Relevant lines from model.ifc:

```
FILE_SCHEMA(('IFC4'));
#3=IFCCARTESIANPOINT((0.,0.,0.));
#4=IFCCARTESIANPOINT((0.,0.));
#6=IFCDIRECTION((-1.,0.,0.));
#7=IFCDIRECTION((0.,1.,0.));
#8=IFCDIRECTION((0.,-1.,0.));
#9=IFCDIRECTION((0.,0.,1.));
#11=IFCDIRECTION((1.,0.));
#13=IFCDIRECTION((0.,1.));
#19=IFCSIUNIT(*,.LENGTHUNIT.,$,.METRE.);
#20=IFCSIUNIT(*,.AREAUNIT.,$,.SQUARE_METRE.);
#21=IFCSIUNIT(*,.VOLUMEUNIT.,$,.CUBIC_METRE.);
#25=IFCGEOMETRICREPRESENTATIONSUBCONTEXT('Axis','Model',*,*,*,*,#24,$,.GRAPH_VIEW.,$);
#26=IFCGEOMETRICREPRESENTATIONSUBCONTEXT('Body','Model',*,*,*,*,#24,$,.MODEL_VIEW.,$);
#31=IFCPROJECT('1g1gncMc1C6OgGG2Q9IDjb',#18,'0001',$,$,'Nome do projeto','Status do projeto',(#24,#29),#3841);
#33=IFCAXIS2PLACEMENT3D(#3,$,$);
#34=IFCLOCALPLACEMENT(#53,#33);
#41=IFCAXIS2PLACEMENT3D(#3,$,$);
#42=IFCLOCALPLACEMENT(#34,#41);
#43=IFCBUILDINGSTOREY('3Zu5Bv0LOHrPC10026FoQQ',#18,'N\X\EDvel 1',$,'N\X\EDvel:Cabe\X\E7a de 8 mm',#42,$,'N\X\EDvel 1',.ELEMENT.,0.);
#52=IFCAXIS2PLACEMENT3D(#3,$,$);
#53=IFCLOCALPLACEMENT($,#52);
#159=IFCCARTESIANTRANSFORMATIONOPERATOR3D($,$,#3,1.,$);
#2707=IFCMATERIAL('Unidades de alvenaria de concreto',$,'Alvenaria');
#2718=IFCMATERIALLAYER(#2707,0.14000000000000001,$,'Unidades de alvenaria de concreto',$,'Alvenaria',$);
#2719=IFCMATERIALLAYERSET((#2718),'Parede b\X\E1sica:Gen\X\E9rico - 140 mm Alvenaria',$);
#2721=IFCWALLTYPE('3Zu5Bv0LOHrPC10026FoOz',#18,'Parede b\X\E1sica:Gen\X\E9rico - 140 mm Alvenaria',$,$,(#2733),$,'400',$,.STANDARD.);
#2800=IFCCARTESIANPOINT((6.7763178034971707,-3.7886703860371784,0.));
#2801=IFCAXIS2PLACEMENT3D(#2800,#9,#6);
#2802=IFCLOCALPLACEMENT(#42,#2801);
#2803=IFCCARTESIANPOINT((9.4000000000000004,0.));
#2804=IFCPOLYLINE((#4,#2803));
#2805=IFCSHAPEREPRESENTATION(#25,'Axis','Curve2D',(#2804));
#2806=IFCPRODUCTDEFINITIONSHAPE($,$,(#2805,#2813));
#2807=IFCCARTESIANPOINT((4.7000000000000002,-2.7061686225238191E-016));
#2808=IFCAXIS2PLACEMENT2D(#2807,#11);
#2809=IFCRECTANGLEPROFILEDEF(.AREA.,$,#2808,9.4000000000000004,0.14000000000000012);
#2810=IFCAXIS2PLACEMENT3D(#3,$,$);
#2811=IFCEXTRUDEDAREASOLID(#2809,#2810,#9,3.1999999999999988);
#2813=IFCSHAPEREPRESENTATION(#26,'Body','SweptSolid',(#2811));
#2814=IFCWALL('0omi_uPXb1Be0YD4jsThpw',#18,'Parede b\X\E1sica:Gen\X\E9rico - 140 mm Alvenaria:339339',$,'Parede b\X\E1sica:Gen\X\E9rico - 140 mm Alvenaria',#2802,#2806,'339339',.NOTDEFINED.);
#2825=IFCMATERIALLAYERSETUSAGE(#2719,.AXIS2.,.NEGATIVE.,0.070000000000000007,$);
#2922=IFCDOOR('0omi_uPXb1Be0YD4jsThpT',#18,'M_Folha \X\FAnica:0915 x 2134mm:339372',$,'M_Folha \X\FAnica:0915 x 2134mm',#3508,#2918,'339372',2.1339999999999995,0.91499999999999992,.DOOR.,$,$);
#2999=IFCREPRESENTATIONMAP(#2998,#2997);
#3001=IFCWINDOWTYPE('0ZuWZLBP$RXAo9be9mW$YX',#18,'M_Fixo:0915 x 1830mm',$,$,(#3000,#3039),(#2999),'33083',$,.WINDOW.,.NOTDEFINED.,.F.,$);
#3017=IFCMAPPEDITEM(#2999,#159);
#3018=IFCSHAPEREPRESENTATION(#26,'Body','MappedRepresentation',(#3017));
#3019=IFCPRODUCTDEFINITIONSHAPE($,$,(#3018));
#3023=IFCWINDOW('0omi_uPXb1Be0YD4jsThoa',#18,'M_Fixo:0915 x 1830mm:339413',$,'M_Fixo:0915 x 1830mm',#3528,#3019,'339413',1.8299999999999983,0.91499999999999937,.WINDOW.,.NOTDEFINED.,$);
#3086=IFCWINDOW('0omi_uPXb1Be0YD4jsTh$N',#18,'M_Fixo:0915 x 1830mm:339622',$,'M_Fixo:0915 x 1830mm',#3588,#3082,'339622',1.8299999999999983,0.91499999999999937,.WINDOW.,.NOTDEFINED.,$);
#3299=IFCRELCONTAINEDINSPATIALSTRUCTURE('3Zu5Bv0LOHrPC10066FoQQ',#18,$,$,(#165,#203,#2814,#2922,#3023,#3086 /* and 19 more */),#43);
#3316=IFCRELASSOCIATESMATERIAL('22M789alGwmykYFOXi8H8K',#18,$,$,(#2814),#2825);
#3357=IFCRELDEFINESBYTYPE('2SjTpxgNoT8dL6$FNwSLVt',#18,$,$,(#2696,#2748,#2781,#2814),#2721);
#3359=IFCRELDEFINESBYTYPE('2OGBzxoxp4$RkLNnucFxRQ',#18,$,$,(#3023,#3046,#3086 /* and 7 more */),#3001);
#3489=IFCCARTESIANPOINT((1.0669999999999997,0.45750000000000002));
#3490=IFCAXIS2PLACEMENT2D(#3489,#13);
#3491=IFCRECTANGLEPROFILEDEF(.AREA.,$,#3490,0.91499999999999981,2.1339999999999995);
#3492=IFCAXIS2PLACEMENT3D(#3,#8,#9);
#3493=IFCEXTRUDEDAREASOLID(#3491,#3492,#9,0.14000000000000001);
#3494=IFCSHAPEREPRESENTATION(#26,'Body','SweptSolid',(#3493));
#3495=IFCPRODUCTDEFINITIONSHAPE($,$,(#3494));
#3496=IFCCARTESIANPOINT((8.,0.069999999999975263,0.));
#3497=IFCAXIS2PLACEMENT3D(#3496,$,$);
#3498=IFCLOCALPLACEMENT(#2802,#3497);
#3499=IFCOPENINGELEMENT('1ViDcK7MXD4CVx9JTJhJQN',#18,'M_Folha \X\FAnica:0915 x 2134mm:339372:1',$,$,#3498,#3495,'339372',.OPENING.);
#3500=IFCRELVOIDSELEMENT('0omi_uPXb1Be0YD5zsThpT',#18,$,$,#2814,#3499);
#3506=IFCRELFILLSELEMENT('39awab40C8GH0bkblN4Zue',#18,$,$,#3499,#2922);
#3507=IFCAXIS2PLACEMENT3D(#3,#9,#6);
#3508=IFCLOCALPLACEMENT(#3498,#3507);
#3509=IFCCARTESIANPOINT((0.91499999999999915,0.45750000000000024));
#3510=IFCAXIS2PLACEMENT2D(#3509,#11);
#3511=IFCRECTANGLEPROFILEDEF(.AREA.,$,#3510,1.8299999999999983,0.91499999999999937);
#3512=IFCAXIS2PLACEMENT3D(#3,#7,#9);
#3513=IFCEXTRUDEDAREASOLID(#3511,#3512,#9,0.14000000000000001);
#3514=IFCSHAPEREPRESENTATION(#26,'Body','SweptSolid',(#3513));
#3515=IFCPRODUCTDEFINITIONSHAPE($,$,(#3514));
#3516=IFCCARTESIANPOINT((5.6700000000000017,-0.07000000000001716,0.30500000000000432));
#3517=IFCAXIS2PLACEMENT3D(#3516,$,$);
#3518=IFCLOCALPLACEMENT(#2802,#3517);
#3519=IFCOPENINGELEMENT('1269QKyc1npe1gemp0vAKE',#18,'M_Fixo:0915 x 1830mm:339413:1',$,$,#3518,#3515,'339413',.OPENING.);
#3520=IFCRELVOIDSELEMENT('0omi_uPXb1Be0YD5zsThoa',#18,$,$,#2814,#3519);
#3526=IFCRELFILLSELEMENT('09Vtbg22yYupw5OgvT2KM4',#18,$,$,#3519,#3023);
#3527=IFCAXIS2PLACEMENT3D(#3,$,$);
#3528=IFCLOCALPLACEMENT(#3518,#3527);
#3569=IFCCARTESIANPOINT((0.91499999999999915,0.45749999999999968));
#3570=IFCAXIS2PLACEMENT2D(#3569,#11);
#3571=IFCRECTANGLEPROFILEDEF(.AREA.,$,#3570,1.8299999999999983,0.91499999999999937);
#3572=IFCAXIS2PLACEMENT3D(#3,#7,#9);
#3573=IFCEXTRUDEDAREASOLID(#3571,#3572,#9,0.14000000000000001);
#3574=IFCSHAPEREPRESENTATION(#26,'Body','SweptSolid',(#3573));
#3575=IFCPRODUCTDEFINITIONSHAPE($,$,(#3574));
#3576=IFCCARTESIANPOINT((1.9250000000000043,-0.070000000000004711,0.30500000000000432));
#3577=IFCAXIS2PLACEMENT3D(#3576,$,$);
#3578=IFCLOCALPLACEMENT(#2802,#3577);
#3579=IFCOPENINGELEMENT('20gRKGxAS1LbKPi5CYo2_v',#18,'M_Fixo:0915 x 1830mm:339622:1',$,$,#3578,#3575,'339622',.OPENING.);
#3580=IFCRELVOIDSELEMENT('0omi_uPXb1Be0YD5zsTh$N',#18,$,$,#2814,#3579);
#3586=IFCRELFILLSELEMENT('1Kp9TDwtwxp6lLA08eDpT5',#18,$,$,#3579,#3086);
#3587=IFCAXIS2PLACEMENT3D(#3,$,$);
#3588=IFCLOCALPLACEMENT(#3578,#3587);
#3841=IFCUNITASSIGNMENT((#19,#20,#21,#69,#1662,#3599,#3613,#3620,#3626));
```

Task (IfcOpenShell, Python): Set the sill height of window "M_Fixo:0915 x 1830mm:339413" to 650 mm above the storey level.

```python
import numpy as np
import ifcopenshell
import ifcopenshell.api.geometry
import ifcopenshell.geom
import ifcopenshell.util.element
import ifcopenshell.util.placement
import ifcopenshell.util.shape
import ifcopenshell.util.unit

model = ifcopenshell.open("model.ifc")
unit_scale = ifcopenshell.util.unit.calculate_unit_scale(model)

window = model.by_guid("0omi_uPXb1Be0YD4jsThoa")
opening = window.FillsVoids[0].RelatingOpeningElement
storey = ifcopenshell.util.element.get_container(window, ifc_class="IfcBuildingStorey")
level = ifcopenshell.util.placement.get_local_placement(storey.ObjectPlacement)[2, 3]

# The opening's origin need not be at the sill, so measure its lowest point.
shape = ifcopenshell.geom.create_shape(ifcopenshell.geom.settings(), opening)
bottom = ifcopenshell.util.shape.get_shape_bottom_elevation(shape, shape.geometry) / unit_scale
dz = level + 0.65 / unit_scale - bottom

shift = np.array([0.0, 0.0, dz])
# The window is placed relative to its opening, so it follows when the opening moves.
matrix = ifcopenshell.util.placement.get_local_placement(opening.ObjectPlacement)
matrix[:3, 3] += shift
ifcopenshell.api.geometry.edit_object_placement(
    model, product=opening, matrix=matrix, is_si=False, should_transform_children=True
)

print(f"moved by {dz * unit_scale:+.3f} m")

model.write("model_edited.ifc")
```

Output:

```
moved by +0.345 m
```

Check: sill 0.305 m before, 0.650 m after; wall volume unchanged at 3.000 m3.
